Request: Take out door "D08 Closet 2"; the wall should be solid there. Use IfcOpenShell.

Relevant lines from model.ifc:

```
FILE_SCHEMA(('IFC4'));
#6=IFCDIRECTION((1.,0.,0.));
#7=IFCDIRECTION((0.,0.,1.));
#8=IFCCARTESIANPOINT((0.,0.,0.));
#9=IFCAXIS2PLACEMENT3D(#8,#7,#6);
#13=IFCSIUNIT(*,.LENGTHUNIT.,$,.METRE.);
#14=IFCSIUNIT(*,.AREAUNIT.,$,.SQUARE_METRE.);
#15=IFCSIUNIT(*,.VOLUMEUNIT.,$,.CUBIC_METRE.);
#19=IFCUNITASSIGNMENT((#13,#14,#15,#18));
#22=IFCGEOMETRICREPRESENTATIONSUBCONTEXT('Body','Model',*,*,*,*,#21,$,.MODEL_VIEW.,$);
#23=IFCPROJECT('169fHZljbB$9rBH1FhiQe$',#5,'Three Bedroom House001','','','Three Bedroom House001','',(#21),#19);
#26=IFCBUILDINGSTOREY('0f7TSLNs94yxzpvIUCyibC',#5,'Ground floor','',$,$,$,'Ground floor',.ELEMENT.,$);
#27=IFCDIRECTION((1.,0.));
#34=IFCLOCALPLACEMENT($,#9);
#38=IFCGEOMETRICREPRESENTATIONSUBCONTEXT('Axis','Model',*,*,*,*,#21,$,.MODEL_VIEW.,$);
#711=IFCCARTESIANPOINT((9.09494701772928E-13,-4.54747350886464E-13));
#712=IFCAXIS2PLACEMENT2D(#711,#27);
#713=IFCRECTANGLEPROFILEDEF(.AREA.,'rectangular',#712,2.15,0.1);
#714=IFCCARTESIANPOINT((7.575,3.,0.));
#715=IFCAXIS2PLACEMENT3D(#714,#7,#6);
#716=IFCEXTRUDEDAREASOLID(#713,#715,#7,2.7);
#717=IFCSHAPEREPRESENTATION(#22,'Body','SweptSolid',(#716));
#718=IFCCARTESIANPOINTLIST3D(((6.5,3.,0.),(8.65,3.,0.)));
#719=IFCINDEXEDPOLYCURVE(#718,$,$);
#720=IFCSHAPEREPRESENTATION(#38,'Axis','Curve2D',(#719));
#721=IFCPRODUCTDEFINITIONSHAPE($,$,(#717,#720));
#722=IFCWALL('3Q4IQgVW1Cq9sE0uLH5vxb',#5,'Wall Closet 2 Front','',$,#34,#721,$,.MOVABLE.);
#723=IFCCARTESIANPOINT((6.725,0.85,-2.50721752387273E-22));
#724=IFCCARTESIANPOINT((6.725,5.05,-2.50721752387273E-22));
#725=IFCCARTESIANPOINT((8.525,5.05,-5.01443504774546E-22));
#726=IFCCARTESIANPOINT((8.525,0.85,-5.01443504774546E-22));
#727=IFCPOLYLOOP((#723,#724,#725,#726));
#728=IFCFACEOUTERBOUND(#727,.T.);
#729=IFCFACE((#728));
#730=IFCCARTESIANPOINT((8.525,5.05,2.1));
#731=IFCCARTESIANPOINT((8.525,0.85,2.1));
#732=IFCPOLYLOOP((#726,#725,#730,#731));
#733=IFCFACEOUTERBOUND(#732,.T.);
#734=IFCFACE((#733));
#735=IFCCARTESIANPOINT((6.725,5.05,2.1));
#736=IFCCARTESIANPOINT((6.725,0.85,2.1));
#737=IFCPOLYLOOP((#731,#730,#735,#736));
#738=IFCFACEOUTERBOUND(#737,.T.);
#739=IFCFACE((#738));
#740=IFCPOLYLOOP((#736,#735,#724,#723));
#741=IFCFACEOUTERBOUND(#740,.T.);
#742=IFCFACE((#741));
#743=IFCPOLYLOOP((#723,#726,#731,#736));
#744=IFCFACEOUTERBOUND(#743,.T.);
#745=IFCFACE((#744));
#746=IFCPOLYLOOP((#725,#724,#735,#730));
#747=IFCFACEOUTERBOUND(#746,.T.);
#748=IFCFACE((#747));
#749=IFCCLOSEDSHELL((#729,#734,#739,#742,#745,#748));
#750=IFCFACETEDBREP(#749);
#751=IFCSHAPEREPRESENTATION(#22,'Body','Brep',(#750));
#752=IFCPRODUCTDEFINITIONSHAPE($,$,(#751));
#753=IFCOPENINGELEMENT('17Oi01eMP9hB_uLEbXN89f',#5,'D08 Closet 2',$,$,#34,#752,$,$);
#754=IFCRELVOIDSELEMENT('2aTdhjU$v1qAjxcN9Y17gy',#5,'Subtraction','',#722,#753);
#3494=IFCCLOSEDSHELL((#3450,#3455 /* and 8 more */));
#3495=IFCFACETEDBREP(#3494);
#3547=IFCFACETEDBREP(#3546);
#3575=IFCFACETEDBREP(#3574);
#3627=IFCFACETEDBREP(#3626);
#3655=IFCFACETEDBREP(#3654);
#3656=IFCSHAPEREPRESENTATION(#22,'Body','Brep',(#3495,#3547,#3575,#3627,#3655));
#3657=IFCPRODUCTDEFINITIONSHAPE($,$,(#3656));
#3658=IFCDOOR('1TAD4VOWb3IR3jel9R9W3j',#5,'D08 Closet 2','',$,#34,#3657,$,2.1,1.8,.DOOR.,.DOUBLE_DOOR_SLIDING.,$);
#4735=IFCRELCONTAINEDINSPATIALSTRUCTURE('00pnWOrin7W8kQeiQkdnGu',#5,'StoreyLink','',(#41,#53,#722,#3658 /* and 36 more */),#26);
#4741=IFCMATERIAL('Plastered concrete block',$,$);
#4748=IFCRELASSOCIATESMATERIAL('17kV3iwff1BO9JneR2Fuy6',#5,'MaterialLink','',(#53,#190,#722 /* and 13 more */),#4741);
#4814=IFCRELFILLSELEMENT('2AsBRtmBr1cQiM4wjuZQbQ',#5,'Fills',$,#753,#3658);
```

```python
import ifcopenshell
import ifcopenshell.api.feature
import ifcopenshell.api.root
import ifcopenshell.geom
import ifcopenshell.util.shape

model = ifcopenshell.open("model.ifc")
settings = ifcopenshell.geom.settings()


def volume(element):
    """Net volume in cubic metres, openings subtracted."""
    shape = ifcopenshell.geom.create_shape(settings, element)
    return ifcopenshell.util.shape.get_volume(shape.geometry)


door = model.by_guid("1TAD4VOWb3IR3jel9R9W3j")
opening = door.FillsVoids[0].RelatingOpeningElement
wall = opening.VoidsElements[0].RelatingBuildingElement
before = volume(wall)

ifcopenshell.api.root.remove_product(model, product=door)
ifcopenshell.api.feature.remove_feature(model, feature=opening)

after = volume(wall)

print(f"wall volume {before:.3f} -> {after:.3f} m3")

model.write("model_v2.ifc")
```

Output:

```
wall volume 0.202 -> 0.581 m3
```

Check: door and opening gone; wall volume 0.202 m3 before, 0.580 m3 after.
